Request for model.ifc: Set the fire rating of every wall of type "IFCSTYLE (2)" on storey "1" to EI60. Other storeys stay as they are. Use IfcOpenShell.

First a look at what the model holds.

```python
import ifcopenshell
import ifcopenshell.util.element

model = ifcopenshell.open("model.ifc")
print(model.schema)
storey = next(s for s in model.by_type("IfcBuildingStorey") if s.Name == "1")
walls = [e for e in ifcopenshell.util.element.get_decomposition(storey) if e.is_a("IfcWall")]
seen = {}
for e in walls:
    element_type = ifcopenshell.util.element.get_type(e)
    key = (element_type.Name if element_type != e and element_type else None, ifcopenshell.util.element.get_pset(e, "Pset_WallCommon", "FireRating"))
    seen[key] = seen.get(key, 0) + 1
for (name, value), count in sorted(seen.items(), key=str):
    print(count, "x", name, "|", value)
```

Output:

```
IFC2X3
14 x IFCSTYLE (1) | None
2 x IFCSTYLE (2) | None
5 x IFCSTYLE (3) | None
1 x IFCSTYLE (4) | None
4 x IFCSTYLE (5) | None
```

```python
import ifcopenshell
import ifcopenshell.api.pset
import ifcopenshell.util.element

model = ifcopenshell.open("model.ifc")

storey = next(s for s in model.by_type("IfcBuildingStorey") if s.Name == "1")
walls = [e for e in ifcopenshell.util.element.get_decomposition(storey) if e.is_a("IfcWall")]

count = 0
for e in walls:
    element_type = ifcopenshell.util.element.get_type(e)
    if element_type in (None, e) or element_type.Name != "IFCSTYLE (2)":
        continue
    # add_pset returns the element's existing set when there is one.
    pset = ifcopenshell.api.pset.add_pset(model, product=e, name="Pset_WallCommon")
    ifcopenshell.api.pset.edit_pset(model, pset=pset, properties={"FireRating": "EI60"})
    count += 1

print(count, "walls updated")

model.write("model_v2.ifc")
```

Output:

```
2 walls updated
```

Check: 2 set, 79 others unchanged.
